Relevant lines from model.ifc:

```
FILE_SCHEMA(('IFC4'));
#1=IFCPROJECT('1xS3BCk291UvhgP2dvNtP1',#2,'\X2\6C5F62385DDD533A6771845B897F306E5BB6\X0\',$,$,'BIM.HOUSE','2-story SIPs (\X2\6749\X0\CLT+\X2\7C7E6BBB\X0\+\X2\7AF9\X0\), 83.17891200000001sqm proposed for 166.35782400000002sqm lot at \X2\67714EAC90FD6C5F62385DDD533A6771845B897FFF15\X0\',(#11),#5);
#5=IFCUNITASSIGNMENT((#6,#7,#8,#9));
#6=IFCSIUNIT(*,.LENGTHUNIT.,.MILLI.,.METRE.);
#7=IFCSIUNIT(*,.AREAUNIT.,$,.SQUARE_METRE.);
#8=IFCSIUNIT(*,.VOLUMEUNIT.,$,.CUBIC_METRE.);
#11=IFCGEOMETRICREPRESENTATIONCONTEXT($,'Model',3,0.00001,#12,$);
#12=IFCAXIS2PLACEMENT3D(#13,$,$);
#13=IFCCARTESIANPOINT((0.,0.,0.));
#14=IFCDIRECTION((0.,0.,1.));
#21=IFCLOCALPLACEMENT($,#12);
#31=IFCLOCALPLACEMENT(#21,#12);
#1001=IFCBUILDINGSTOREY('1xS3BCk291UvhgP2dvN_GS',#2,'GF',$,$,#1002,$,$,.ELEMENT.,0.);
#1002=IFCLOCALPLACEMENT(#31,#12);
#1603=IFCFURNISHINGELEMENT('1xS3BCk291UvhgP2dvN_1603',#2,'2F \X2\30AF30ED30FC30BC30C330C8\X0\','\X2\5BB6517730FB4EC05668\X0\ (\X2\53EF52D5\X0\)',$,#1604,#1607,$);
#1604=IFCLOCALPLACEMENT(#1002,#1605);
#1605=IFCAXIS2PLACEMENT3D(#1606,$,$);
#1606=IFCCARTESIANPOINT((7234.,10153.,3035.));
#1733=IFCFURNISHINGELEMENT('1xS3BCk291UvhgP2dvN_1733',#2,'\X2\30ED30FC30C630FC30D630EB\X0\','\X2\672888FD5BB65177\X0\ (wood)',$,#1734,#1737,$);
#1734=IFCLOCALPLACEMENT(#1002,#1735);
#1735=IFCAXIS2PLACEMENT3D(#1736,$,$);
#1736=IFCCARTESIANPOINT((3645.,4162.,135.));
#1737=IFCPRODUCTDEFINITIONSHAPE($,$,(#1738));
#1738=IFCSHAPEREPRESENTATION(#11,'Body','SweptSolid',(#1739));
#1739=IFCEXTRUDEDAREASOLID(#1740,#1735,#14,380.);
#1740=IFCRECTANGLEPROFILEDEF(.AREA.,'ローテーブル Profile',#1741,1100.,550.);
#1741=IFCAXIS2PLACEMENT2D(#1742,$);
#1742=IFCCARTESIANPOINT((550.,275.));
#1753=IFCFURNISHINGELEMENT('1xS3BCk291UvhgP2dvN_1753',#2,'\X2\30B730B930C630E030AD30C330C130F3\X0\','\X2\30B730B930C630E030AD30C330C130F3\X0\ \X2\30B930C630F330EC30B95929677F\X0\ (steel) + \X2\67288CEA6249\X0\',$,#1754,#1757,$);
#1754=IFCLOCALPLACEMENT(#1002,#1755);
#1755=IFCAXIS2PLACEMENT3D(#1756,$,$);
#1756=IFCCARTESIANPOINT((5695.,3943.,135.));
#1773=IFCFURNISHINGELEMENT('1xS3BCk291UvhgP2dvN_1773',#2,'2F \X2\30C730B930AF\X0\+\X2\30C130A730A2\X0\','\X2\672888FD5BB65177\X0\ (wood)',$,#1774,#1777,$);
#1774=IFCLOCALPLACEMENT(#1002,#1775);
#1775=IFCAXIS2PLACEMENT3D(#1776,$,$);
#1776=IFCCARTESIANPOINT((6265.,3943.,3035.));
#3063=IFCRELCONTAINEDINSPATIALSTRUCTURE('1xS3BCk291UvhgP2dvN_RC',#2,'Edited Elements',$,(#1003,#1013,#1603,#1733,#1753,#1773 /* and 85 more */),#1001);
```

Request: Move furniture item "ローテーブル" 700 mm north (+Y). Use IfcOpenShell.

```python
import ifcopenshell
import ifcopenshell.api.geometry
import ifcopenshell.util.placement
import ifcopenshell.util.unit

model = ifcopenshell.open("model.ifc")
unit_scale = ifcopenshell.util.unit.calculate_unit_scale(model)

item = model.by_guid("1xS3BCk291UvhgP2dvN_1733")
matrix = ifcopenshell.util.placement.get_local_placement(item.ObjectPlacement)
matrix[1, 3] += 0.7 / unit_scale
ifcopenshell.api.geometry.edit_object_placement(model, product=item, matrix=matrix, is_si=False)

print(ifcopenshell.util.placement.get_local_placement(item.ObjectPlacement).round(3) + 0.0)

model.write("model_edited.ifc")
```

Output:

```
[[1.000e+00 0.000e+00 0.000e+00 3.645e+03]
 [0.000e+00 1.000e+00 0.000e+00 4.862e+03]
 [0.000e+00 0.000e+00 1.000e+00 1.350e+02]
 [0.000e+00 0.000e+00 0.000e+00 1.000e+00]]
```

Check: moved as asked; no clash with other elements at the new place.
